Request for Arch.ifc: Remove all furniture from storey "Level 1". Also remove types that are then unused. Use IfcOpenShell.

First a look at what the model holds.

```python
import ifcopenshell
import ifcopenshell.util.element

model = ifcopenshell.open("Arch.ifc")
print(model.schema)
storey = next(s for s in model.by_type("IfcBuildingStorey") if s.Name == "Level 1")
furniture = [e for e in ifcopenshell.util.element.get_decomposition(storey) if e.is_a("IfcFurnishingElement")]
seen = {}
for e in furniture:
    element_type = ifcopenshell.util.element.get_type(e)
    name = element_type.Name if element_type not in (None, e) else None
    seen[name] = seen.get(name, 0) + 1
for name, count in sorted(seen.items(), key=str):
    print(count, "x", name)
```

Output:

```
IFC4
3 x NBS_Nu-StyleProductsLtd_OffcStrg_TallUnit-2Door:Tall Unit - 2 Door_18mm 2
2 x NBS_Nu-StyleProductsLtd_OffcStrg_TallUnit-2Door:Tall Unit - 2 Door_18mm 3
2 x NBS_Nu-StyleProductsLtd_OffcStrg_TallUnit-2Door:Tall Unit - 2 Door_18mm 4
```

```python
import ifcopenshell
import ifcopenshell.api.root
import ifcopenshell.util.element

model = ifcopenshell.open("Arch.ifc")

storey = next(s for s in model.by_type("IfcBuildingStorey") if s.Name == "Level 1")
furniture = [e for e in ifcopenshell.util.element.get_decomposition(storey) if e.is_a("IfcFurnishingElement")]
types = {ifcopenshell.util.element.get_type(e) for e in furniture} - {None, *furniture}

for e in furniture:
    ifcopenshell.api.root.remove_product(model, product=e)
print(len(furniture), "removed")

unused = [t for t in types if not ifcopenshell.util.element.get_types(t)]
for t in unused:
    ifcopenshell.api.root.remove_product(model, product=t)
print(len(unused), "unused types removed")

model.write("Arch-out.ifc")
```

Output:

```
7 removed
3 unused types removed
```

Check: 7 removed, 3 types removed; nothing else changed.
